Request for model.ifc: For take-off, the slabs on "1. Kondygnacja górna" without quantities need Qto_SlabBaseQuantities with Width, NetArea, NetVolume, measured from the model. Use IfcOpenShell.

First a look at what the model holds.

```python
import ifcopenshell
import ifcopenshell.util.element
import ifcopenshell.util.unit

model = ifcopenshell.open("model.ifc")
print(model.schema)
for unit_type in ("LENGTHUNIT", "AREAUNIT", "VOLUMEUNIT"):
    print(unit_type, ifcopenshell.util.unit.calculate_unit_scale(model, unit_type))
storey = next(s for s in model.by_type("IfcBuildingStorey") if s.Name == "1. Kondygnacja górna")
slabs = [e for e in ifcopenshell.util.element.get_decomposition(storey) if e.is_a("IfcSlab")]
for e in sorted(slabs, key=lambda e: e.id()):
    print(e.id(), e.is_a(), e.Name, list(ifcopenshell.util.element.get_psets(e, qtos_only=True)), sep=" | ")
```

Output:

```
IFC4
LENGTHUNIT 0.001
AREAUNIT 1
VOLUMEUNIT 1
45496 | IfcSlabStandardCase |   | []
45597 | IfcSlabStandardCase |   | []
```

```python
import ifcopenshell
import ifcopenshell.api.pset
import ifcopenshell.geom
import ifcopenshell.util.element
import ifcopenshell.util.shape
import ifcopenshell.util.unit

model = ifcopenshell.open("model.ifc")
unit_scale = ifcopenshell.util.unit.calculate_unit_scale(model)
area_scale = ifcopenshell.util.unit.calculate_unit_scale(model, "AREAUNIT")
volume_scale = ifcopenshell.util.unit.calculate_unit_scale(model, "VOLUMEUNIT")
settings = ifcopenshell.geom.settings()

storey = next(s for s in model.by_type("IfcBuildingStorey") if s.Name == "1. Kondygnacja górna")
slabs = [e for e in ifcopenshell.util.element.get_decomposition(storey) if e.is_a("IfcSlab")]

for e in sorted(slabs, key=lambda e: e.id()):
    if ifcopenshell.util.element.get_psets(e, qtos_only=True, should_inherit=False):
        continue
    # Geometry comes back in metres, in the element's own axes.
    shape = ifcopenshell.geom.create_shape(settings, e)
    values = {
        "Width": ifcopenshell.util.shape.get_z(shape.geometry) / unit_scale,
        "NetArea": ifcopenshell.util.shape.get_footprint_area(shape.geometry) / area_scale,
        "NetVolume": ifcopenshell.util.shape.get_volume(shape.geometry) / volume_scale,
    }
    qto = ifcopenshell.api.pset.add_qto(model, product=e, name="Qto_SlabBaseQuantities")
    ifcopenshell.api.pset.edit_qto(model, qto=qto, properties=values)
    print(e.id(), {k: round(v, 3) for k, v in values.items()})

model.write("model_edited.ifc")
```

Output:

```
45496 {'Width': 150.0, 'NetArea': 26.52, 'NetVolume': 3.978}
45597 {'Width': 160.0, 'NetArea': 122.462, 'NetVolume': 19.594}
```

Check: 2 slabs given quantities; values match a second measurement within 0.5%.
